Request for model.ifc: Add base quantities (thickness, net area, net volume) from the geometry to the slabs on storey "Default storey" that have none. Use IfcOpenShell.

First a look at what the model holds.

```python
import ifcopenshell
import ifcopenshell.util.element
import ifcopenshell.util.unit

model = ifcopenshell.open("model.ifc")
print(model.schema)
for unit_type in ("LENGTHUNIT", "AREAUNIT", "VOLUMEUNIT"):
    print(unit_type, ifcopenshell.util.unit.calculate_unit_scale(model, unit_type))
storey = next(s for s in model.by_type("IfcBuildingStorey") if s.Name == "Default storey")
slabs = [e for e in ifcopenshell.util.element.get_decomposition(storey) if e.is_a("IfcSlab")]
for e in sorted(slabs, key=lambda e: e.id()):
    print(e.id(), e.is_a(), e.Name, list(ifcopenshell.util.element.get_psets(e, qtos_only=True)), sep=" | ")
```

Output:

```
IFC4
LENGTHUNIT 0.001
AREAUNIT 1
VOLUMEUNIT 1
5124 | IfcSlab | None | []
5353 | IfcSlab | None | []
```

```python
import ifcopenshell
import ifcopenshell.api.pset
import ifcopenshell.geom
import ifcopenshell.util.element
import ifcopenshell.util.shape
import ifcopenshell.util.unit

model = ifcopenshell.open("model.ifc")
unit_scale = ifcopenshell.util.unit.calculate_unit_scale(model)
area_scale = ifcopenshell.util.unit.calculate_unit_scale(model, "AREAUNIT")
volume_scale = ifcopenshell.util.unit.calculate_unit_scale(model, "VOLUMEUNIT")
settings = ifcopenshell.geom.settings()

storey = next(s for s in model.by_type("IfcBuildingStorey") if s.Name == "Default storey")
slabs = [e for e in ifcopenshell.util.element.get_decomposition(storey) if e.is_a("IfcSlab")]

for e in sorted(slabs, key=lambda e: e.id()):
    if ifcopenshell.util.element.get_psets(e, qtos_only=True, should_inherit=False):
        continue
    # Geometry comes back in metres, in the element's own axes.
    shape = ifcopenshell.geom.create_shape(settings, e)
    values = {
        "Width": ifcopenshell.util.shape.get_z(shape.geometry) / unit_scale,
        "NetArea": ifcopenshell.util.shape.get_footprint_area(shape.geometry) / area_scale,
        "NetVolume": ifcopenshell.util.shape.get_volume(shape.geometry) / volume_scale,
    }
    qto = ifcopenshell.api.pset.add_qto(model, product=e, name="Qto_SlabBaseQuantities")
    ifcopenshell.api.pset.edit_qto(model, qto=qto, properties=values)
    print(e.id(), {k: round(v, 3) for k, v in values.items()})

model.write("model-out.ifc")
```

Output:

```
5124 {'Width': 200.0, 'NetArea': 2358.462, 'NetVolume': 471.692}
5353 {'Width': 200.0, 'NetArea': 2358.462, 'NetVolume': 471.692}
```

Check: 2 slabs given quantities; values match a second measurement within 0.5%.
